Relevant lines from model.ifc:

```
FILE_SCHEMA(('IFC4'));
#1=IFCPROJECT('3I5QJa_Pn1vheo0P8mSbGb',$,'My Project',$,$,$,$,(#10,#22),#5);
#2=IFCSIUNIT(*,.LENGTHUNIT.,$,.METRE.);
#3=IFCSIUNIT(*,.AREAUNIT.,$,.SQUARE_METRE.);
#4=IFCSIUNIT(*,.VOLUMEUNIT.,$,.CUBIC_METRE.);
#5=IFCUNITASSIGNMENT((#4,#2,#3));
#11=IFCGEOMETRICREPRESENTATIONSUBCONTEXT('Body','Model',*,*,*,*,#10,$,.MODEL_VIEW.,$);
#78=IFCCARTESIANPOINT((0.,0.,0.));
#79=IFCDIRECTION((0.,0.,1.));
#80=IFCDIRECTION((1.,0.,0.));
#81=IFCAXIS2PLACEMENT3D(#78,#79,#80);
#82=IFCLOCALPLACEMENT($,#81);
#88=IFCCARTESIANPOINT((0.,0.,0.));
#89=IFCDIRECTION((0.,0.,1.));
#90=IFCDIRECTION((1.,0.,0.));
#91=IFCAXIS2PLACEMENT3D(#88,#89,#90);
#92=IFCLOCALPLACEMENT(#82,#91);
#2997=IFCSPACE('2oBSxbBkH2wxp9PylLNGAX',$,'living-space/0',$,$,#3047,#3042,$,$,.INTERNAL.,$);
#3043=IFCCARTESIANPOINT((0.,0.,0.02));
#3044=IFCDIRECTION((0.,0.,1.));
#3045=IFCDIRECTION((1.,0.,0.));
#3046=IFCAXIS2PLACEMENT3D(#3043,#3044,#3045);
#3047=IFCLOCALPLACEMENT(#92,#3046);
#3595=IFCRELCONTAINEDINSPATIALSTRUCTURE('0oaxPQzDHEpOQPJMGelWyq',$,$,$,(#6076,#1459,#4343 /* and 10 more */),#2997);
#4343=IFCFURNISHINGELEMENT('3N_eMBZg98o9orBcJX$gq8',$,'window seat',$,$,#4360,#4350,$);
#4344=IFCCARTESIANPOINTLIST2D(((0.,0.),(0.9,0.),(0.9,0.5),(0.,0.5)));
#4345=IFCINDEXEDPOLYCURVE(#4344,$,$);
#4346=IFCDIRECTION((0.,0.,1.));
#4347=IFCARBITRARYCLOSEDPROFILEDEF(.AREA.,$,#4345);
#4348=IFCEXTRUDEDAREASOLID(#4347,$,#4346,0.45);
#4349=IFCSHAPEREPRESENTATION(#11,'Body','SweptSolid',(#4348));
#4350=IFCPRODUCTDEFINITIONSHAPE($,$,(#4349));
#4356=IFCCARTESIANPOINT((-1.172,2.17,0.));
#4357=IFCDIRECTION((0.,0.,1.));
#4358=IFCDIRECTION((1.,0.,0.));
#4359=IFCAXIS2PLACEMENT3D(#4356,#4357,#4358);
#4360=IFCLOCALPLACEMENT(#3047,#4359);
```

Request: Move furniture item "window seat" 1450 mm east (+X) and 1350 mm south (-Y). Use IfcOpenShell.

```python
import ifcopenshell
import ifcopenshell.api.geometry
import ifcopenshell.util.placement

model = ifcopenshell.open("model.ifc")

item = model.by_guid("3N_eMBZg98o9orBcJX$gq8")
matrix = ifcopenshell.util.placement.get_local_placement(item.ObjectPlacement)
matrix[0, 3] += 1.45
matrix[1, 3] -= 1.35
ifcopenshell.api.geometry.edit_object_placement(model, product=item, matrix=matrix, is_si=False)

print(ifcopenshell.util.placement.get_local_placement(item.ObjectPlacement).round(3) + 0.0)

model.write("model_edited.ifc")
```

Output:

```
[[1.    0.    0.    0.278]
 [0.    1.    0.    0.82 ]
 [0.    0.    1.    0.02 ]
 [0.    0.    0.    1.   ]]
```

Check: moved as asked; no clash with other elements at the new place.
